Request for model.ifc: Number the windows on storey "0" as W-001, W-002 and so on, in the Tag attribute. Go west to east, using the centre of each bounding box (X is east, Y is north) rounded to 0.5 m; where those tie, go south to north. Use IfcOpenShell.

First a look at what the model holds.

```python
import ifcopenshell
import ifcopenshell.util.element
import ifcopenshell.util.placement

model = ifcopenshell.open("model.ifc")
print(model.schema)
storey = next(s for s in model.by_type("IfcBuildingStorey") if s.Name == "0")
windows = [e for e in ifcopenshell.util.element.get_decomposition(storey) if e.is_a("IfcWindow")]
for e in sorted(windows, key=lambda e: e.id()):
    origin = ifcopenshell.util.placement.get_local_placement(e.ObjectPlacement)[:3, 3]
    print(e.id(), e.Tag, e.Name, origin.round(2) + 0.0, sep=" | ")
```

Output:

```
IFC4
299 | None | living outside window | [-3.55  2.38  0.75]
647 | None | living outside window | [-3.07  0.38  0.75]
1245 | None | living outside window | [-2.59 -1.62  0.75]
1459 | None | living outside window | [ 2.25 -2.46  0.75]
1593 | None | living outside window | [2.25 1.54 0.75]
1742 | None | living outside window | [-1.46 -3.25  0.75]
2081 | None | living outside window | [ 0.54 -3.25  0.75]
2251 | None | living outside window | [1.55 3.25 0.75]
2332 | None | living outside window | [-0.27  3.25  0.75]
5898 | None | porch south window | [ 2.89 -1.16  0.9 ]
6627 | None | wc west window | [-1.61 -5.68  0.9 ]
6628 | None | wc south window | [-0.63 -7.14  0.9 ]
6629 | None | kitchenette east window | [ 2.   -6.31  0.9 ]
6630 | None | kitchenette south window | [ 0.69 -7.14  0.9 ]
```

```python
import ifcopenshell
import ifcopenshell.geom
import ifcopenshell.util.element
import ifcopenshell.util.shape

model = ifcopenshell.open("model.ifc")
settings = ifcopenshell.geom.settings()
settings.set("use-world-coords", True)


def centre(element):
    shape = ifcopenshell.geom.create_shape(settings, element)
    return ifcopenshell.util.shape.get_bbox_centroid(shape.geometry)


storey = next(s for s in model.by_type("IfcBuildingStorey") if s.Name == "0")
windows = [e for e in ifcopenshell.util.element.get_decomposition(storey) if e.is_a("IfcWindow")]

# Insertion points can sit at a corner or the storey origin, so sort by the geometry (in metres).
centres = {e: centre(e) for e in windows}
windows.sort(key=lambda e: (round(centres[e][0] / 0.5), centres[e][1]))

for i, e in enumerate(windows, start=1):
    number = f"W-0{i:02d}"
    e.Tag = number
    print(e.id(), number)

model.write("model_updated.ifc")
```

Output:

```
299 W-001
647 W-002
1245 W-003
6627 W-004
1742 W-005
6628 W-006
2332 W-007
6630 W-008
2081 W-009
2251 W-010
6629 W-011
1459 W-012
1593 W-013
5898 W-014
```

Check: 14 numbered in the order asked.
